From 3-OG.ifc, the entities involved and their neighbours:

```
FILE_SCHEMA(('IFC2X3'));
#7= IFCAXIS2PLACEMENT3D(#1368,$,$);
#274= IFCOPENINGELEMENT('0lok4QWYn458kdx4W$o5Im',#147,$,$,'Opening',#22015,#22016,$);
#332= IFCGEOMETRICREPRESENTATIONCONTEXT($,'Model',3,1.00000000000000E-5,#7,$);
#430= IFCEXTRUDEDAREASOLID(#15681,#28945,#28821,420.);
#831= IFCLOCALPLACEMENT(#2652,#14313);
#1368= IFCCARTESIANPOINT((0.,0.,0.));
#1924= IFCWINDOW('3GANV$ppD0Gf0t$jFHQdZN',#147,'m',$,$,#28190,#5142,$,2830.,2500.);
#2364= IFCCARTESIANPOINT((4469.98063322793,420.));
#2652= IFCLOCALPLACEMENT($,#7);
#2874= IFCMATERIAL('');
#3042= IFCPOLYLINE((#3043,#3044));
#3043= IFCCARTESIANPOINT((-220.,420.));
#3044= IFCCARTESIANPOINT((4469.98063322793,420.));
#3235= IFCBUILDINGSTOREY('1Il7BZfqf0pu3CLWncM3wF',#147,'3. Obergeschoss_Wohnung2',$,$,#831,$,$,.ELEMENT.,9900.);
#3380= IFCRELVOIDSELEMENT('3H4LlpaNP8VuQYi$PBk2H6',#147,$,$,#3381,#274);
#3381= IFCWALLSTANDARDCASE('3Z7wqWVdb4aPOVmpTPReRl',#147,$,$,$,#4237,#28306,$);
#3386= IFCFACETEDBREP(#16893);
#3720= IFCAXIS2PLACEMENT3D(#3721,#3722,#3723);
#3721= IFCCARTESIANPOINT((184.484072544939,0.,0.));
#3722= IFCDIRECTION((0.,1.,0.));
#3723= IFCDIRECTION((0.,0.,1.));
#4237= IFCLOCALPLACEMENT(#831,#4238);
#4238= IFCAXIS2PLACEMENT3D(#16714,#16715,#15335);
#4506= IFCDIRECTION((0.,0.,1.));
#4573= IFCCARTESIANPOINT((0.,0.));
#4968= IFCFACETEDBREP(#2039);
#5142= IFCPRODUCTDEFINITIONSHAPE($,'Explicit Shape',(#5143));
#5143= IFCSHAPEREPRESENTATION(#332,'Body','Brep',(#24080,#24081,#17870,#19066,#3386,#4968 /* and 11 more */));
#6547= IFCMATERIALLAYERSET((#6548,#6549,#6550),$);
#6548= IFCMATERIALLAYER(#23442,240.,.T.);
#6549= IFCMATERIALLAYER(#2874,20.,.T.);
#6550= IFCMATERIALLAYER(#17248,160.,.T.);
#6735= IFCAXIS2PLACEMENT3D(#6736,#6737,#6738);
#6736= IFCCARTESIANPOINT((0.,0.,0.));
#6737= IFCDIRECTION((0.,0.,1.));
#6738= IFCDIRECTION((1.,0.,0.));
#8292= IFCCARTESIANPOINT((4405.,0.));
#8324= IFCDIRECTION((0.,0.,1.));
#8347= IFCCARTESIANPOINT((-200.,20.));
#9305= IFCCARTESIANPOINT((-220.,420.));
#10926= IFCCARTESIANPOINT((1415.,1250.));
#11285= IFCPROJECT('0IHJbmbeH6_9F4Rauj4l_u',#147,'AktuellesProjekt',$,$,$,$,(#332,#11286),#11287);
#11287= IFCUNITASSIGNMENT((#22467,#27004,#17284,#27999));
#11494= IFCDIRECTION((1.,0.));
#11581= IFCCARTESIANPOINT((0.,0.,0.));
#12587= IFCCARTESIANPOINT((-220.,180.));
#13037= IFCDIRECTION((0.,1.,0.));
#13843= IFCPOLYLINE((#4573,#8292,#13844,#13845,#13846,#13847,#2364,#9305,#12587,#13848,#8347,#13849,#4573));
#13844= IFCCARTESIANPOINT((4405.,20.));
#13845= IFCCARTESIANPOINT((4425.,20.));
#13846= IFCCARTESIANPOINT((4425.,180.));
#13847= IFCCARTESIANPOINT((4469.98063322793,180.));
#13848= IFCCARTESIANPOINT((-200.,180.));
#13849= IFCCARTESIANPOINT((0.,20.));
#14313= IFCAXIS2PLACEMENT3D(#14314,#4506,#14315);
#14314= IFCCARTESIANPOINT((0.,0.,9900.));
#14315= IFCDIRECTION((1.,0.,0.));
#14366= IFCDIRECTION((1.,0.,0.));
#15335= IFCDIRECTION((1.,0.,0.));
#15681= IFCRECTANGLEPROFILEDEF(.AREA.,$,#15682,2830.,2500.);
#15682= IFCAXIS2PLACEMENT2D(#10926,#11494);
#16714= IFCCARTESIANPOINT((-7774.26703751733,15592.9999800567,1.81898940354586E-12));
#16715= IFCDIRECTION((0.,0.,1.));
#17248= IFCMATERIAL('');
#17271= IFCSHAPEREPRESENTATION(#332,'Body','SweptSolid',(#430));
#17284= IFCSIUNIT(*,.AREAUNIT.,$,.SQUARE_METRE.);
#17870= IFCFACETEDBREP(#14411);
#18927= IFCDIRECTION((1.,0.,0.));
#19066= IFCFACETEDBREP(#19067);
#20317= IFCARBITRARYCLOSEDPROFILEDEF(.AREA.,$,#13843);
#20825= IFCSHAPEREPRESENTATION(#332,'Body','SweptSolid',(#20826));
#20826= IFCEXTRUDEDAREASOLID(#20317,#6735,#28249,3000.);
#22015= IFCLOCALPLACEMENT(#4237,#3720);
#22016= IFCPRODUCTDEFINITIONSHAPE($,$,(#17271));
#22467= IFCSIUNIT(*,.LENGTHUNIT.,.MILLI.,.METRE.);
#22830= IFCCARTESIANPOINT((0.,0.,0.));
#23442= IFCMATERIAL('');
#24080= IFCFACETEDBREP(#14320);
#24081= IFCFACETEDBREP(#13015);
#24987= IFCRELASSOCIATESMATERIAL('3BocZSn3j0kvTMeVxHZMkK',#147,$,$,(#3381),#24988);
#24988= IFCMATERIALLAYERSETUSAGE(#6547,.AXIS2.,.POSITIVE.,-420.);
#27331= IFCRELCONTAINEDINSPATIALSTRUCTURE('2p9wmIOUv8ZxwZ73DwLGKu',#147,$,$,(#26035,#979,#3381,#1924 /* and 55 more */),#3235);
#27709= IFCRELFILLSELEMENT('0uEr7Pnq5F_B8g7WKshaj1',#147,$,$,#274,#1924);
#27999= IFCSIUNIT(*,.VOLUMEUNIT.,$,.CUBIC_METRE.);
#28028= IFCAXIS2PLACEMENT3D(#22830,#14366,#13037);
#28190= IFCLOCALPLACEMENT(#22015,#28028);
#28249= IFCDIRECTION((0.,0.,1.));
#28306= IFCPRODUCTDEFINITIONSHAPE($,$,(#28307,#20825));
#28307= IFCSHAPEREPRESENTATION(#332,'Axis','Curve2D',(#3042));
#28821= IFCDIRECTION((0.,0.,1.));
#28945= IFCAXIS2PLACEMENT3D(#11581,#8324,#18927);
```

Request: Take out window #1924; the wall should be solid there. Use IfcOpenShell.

```python
import ifcopenshell
import ifcopenshell.api.feature
import ifcopenshell.api.root
import ifcopenshell.geom
import ifcopenshell.util.shape

model = ifcopenshell.open("3-OG.ifc")
settings = ifcopenshell.geom.settings()


def volume(element):
    """Net volume in cubic metres, openings subtracted."""
    shape = ifcopenshell.geom.create_shape(settings, element)
    return ifcopenshell.util.shape.get_volume(shape.geometry)


window = model.by_id(1924)
opening = window.FillsVoids[0].RelatingOpeningElement
wall = opening.VoidsElements[0].RelatingBuildingElement
before = volume(wall)

ifcopenshell.api.root.remove_product(model, product=window)
ifcopenshell.api.feature.remove_feature(model, feature=opening)

after = volume(wall)

print(f"wall volume {before:.3f} -> {after:.3f} m3")

model.write("3-OG-out.ifc")
```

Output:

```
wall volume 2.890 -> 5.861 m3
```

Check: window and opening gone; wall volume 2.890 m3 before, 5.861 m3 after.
